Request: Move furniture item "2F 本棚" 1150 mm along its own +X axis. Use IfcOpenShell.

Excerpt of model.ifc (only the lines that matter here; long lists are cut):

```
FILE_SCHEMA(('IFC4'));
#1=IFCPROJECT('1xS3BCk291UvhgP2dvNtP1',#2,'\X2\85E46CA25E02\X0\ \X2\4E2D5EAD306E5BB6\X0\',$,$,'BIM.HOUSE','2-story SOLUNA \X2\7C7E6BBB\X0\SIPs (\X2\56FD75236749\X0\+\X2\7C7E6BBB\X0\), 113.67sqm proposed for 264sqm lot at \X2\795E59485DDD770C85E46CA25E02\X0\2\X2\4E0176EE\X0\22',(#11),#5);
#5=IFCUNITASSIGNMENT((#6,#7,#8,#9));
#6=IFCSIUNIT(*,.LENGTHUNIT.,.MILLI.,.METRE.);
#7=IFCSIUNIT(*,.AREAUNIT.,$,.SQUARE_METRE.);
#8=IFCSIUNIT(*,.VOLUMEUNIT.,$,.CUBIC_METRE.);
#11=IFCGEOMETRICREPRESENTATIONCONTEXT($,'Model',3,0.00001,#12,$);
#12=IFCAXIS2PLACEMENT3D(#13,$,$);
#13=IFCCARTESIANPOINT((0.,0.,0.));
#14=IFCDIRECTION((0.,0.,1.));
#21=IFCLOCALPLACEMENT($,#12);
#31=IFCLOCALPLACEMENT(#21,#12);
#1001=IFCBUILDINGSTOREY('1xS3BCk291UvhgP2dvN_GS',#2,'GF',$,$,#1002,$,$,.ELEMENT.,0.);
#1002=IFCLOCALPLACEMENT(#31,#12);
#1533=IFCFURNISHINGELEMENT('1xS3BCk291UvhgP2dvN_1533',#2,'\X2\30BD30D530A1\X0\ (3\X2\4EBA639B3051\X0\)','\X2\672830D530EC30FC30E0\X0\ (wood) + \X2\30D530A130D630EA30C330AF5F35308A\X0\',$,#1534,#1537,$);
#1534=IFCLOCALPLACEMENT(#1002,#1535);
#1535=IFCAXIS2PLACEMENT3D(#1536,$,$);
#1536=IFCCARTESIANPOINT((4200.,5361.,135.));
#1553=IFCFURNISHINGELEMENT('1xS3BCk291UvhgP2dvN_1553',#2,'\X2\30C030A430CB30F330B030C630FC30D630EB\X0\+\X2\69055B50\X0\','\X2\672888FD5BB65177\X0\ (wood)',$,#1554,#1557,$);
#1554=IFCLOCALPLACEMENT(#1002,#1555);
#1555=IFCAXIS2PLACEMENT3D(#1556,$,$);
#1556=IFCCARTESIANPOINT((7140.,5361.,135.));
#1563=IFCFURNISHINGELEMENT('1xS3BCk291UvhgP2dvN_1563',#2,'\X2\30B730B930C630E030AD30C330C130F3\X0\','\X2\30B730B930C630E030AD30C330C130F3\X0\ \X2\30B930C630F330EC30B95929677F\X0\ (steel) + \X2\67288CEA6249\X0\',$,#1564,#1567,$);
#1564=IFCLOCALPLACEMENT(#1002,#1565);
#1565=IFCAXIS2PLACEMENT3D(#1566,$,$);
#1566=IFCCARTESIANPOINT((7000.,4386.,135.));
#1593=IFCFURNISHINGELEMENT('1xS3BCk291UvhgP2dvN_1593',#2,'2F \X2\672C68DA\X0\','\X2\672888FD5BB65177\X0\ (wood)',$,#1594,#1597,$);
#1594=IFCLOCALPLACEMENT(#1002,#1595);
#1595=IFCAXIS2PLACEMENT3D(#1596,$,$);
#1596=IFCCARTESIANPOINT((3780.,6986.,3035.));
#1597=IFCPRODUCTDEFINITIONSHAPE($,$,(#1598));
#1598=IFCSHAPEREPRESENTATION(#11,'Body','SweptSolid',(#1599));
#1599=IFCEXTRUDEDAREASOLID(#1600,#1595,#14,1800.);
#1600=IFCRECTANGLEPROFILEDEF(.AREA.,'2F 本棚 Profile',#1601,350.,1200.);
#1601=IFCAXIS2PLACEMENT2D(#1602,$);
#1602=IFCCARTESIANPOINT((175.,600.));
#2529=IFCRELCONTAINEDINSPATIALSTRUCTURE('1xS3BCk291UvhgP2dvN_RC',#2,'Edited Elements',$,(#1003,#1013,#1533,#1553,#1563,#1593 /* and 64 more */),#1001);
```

```python
import ifcopenshell
import ifcopenshell.api.geometry
import ifcopenshell.util.placement
import ifcopenshell.util.unit

model = ifcopenshell.open("model.ifc")
unit_scale = ifcopenshell.util.unit.calculate_unit_scale(model)

item = model.by_guid("1xS3BCk291UvhgP2dvN_1593")
matrix = ifcopenshell.util.placement.get_local_placement(item.ObjectPlacement)
matrix[:3, 3] += matrix[:3, 0] * 1.15 / unit_scale
ifcopenshell.api.geometry.edit_object_placement(model, product=item, matrix=matrix, is_si=False)

print(ifcopenshell.util.placement.get_local_placement(item.ObjectPlacement).round(3) + 0.0)

model.write("model_edited.ifc")
```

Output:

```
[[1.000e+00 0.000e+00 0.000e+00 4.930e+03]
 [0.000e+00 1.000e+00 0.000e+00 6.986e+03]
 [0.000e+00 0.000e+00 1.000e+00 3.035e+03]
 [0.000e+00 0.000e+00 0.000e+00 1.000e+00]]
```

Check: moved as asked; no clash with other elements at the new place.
